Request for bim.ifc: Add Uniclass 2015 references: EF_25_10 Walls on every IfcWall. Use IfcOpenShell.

First a look at what the model holds.

```python
import ifcopenshell

model = ifcopenshell.open("bim.ifc")
print(model.schema)
print("classifications:", [c.Name for c in model.by_type("IfcClassification")])
for ifc_class in ("IfcDoor", "IfcRoof", "IfcStair", "IfcWall", "IfcWindow"):
    print(ifc_class, len(model.by_type(ifc_class)))
```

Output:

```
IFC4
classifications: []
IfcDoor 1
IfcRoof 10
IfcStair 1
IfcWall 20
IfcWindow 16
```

```python
import ifcopenshell
import ifcopenshell.api.classification

model = ifcopenshell.open("bim.ifc")

system = ifcopenshell.api.classification.add_classification(model, classification="Uniclass 2015")

codes = {
    "IfcWall": ("EF_25_10", "Walls"),
}
for ifc_class, (code, name) in codes.items():
    products = model.by_type(ifc_class)
    ifcopenshell.api.classification.add_reference(
        model, products=products, classification=system, identification=code, name=name
    )
    print(code, len(products))

model.write("bim_updated.ifc")
```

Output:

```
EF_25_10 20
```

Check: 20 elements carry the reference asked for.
